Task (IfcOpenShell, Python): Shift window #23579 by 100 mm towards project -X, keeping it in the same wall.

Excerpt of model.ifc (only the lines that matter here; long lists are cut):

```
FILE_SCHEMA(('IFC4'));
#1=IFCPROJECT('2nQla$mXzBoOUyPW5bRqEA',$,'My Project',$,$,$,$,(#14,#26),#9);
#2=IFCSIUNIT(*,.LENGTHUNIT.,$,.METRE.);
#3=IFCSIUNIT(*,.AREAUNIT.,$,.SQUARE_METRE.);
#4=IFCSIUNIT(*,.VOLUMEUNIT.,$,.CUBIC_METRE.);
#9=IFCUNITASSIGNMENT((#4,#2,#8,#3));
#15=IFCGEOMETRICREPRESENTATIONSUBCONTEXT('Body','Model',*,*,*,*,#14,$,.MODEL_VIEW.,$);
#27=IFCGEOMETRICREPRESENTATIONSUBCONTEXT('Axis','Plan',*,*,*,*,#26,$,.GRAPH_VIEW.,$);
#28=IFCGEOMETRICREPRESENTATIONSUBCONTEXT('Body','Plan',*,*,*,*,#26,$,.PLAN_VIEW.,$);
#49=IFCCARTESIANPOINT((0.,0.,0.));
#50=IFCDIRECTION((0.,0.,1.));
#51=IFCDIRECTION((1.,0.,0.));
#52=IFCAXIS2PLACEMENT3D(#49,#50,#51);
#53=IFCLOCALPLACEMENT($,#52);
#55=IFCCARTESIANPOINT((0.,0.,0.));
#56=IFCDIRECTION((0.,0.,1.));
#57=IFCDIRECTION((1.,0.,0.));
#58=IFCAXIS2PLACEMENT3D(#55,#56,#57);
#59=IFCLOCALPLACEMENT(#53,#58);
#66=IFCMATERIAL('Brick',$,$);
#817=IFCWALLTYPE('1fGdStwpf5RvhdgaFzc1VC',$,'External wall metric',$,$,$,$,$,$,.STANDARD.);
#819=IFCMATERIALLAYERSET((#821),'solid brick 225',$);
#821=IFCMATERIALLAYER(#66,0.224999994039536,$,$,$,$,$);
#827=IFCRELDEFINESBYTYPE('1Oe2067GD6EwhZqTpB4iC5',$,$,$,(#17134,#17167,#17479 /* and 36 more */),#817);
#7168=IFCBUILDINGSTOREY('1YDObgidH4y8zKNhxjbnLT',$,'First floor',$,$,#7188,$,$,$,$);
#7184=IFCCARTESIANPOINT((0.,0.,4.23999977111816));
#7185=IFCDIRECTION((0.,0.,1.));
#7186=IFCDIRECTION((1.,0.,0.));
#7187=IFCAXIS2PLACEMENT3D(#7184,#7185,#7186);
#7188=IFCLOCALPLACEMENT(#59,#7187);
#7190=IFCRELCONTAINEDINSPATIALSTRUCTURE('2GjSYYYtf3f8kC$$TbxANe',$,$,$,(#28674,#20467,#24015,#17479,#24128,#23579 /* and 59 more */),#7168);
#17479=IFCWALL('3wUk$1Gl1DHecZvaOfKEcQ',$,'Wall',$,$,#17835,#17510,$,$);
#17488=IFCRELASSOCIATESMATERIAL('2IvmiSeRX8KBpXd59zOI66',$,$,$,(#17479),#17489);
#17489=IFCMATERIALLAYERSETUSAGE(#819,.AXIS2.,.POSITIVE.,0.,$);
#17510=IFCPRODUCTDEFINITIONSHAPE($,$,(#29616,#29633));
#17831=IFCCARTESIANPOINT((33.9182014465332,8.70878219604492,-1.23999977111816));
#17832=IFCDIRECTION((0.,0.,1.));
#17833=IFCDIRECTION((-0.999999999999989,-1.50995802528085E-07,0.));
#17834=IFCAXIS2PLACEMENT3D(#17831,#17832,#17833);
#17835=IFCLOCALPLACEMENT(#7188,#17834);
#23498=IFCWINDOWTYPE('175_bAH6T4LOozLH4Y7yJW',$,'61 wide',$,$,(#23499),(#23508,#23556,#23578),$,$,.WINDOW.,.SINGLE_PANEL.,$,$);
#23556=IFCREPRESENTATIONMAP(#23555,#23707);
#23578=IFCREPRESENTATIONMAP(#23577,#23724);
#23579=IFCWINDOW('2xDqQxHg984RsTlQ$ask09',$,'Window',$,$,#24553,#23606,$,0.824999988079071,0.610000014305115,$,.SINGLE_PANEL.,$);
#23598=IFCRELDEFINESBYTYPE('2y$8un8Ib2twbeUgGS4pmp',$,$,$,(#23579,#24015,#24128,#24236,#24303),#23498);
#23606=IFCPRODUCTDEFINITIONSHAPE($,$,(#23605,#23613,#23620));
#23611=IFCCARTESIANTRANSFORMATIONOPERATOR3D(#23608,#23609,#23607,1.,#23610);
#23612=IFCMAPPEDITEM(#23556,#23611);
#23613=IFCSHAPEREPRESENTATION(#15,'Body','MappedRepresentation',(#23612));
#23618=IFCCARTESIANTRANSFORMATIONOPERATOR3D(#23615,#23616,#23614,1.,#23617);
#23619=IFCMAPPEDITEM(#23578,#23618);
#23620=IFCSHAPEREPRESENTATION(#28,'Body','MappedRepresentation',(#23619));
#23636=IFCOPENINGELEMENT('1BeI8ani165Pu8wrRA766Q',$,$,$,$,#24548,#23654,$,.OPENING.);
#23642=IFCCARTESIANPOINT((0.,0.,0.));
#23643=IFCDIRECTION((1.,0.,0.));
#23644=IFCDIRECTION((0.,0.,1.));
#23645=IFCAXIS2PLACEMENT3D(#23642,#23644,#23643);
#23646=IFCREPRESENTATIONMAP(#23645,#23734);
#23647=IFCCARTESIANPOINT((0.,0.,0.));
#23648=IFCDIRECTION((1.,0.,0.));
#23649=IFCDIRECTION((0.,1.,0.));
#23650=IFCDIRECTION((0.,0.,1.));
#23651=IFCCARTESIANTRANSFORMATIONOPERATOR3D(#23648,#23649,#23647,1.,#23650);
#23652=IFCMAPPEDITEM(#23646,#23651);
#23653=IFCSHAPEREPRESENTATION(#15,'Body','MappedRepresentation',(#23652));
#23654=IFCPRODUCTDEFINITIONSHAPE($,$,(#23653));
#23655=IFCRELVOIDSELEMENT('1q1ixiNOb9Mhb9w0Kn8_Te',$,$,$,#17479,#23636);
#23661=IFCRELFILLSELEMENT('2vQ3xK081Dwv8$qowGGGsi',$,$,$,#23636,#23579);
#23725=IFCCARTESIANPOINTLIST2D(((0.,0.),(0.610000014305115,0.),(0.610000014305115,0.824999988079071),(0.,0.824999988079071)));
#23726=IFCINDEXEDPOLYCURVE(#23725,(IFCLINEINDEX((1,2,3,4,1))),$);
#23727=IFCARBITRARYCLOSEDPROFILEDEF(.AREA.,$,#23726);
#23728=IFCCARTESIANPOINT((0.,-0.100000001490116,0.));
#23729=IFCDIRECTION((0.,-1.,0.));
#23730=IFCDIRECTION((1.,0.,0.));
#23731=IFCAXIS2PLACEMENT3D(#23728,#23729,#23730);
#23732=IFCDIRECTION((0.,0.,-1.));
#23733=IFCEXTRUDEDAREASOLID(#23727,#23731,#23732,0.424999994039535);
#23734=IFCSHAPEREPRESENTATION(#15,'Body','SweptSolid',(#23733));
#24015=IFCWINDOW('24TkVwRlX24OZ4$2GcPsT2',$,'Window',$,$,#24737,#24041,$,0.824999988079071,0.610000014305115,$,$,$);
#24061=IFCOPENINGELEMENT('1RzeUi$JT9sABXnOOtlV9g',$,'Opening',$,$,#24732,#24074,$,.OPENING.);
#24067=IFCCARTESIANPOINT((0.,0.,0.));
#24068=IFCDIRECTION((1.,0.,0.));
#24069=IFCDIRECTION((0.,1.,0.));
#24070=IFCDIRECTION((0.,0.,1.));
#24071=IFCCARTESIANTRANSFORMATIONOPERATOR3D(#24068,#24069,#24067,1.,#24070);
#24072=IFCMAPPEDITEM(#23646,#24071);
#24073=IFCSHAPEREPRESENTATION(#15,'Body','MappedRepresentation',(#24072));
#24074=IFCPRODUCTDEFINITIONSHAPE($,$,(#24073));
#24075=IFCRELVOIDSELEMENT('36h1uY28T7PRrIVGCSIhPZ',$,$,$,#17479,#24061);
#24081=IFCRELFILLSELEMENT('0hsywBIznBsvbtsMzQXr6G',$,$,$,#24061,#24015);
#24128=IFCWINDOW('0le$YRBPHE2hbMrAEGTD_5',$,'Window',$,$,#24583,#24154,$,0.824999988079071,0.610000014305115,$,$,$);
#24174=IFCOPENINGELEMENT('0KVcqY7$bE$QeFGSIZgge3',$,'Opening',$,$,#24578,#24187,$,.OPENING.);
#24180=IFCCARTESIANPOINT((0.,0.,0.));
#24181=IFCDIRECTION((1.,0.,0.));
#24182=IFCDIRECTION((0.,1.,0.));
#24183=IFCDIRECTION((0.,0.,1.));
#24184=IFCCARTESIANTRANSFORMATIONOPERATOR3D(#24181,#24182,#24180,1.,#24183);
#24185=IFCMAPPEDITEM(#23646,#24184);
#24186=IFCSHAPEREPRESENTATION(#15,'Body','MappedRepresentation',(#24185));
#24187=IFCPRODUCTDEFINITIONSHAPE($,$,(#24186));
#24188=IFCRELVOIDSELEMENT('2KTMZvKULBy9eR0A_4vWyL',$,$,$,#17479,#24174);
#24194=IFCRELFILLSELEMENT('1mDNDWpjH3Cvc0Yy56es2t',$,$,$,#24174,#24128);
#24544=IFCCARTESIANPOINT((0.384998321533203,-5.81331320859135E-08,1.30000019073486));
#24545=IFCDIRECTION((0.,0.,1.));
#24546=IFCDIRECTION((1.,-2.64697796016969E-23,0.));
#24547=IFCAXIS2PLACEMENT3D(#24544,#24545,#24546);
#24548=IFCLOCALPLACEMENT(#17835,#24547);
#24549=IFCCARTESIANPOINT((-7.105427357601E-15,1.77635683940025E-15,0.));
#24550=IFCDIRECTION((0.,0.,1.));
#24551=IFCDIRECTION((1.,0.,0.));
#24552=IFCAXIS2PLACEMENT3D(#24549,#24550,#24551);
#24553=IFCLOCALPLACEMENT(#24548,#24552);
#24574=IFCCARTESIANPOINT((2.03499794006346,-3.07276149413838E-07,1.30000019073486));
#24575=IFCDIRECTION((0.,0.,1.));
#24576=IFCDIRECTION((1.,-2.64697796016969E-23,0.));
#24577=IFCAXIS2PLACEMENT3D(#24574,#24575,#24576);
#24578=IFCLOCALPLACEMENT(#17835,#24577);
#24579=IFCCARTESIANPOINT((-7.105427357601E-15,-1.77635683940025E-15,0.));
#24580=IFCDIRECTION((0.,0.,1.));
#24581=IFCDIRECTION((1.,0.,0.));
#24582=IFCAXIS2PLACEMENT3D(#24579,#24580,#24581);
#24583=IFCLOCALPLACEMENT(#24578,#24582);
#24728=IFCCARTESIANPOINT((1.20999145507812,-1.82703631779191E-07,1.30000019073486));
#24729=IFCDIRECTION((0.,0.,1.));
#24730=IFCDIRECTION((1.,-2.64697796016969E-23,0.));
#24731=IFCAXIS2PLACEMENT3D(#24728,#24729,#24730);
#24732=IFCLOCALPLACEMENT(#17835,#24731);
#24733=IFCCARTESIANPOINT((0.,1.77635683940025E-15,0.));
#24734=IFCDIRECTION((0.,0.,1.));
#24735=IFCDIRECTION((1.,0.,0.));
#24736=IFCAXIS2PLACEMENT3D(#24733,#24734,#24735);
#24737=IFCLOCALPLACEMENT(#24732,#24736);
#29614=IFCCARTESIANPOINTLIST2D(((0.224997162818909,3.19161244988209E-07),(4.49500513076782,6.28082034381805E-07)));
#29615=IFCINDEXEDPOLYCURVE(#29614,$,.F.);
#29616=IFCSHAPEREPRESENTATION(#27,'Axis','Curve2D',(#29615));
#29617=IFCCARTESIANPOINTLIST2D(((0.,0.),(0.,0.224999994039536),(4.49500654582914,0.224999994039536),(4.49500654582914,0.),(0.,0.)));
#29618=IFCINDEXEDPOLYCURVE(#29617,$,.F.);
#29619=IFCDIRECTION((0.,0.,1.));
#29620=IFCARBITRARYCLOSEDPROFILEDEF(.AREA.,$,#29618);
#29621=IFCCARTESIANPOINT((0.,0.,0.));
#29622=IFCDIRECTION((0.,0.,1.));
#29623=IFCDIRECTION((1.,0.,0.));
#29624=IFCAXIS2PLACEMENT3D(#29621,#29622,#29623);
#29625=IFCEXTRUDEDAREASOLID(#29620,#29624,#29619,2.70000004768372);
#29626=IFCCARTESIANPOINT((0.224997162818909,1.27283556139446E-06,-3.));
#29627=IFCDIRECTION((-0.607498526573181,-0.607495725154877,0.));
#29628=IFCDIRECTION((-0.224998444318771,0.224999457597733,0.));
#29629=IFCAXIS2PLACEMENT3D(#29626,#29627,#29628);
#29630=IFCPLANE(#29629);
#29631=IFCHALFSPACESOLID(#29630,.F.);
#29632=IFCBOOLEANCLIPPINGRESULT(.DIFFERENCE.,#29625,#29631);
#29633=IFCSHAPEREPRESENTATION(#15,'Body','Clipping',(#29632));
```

```python
import ifcopenshell
import ifcopenshell.api.geometry
import ifcopenshell.util.placement

model = ifcopenshell.open("model.ifc")

window = model.by_id(23579)
opening = window.FillsVoids[0].RelatingOpeningElement
wall = opening.VoidsElements[0].RelatingBuildingElement

wall_matrix = ifcopenshell.util.placement.get_local_placement(wall.ObjectPlacement)
shift = wall_matrix[:3, 0] * 0.1
before = ifcopenshell.util.placement.get_local_placement(window.ObjectPlacement)[:3, 3].copy()

# The window is placed relative to its opening, so it follows when the opening moves.
matrix = ifcopenshell.util.placement.get_local_placement(opening.ObjectPlacement)
matrix[:3, 3] += shift
ifcopenshell.api.geometry.edit_object_placement(
    model, product=opening, matrix=matrix, is_si=False, should_transform_children=True
)

after = ifcopenshell.util.placement.get_local_placement(window.ObjectPlacement)[:3, 3]
print("window moved by", (after - before).round(3) + 0.0)

model.write("model_updated.ifc")
```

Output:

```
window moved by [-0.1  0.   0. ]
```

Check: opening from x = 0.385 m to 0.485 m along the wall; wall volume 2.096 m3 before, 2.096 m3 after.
